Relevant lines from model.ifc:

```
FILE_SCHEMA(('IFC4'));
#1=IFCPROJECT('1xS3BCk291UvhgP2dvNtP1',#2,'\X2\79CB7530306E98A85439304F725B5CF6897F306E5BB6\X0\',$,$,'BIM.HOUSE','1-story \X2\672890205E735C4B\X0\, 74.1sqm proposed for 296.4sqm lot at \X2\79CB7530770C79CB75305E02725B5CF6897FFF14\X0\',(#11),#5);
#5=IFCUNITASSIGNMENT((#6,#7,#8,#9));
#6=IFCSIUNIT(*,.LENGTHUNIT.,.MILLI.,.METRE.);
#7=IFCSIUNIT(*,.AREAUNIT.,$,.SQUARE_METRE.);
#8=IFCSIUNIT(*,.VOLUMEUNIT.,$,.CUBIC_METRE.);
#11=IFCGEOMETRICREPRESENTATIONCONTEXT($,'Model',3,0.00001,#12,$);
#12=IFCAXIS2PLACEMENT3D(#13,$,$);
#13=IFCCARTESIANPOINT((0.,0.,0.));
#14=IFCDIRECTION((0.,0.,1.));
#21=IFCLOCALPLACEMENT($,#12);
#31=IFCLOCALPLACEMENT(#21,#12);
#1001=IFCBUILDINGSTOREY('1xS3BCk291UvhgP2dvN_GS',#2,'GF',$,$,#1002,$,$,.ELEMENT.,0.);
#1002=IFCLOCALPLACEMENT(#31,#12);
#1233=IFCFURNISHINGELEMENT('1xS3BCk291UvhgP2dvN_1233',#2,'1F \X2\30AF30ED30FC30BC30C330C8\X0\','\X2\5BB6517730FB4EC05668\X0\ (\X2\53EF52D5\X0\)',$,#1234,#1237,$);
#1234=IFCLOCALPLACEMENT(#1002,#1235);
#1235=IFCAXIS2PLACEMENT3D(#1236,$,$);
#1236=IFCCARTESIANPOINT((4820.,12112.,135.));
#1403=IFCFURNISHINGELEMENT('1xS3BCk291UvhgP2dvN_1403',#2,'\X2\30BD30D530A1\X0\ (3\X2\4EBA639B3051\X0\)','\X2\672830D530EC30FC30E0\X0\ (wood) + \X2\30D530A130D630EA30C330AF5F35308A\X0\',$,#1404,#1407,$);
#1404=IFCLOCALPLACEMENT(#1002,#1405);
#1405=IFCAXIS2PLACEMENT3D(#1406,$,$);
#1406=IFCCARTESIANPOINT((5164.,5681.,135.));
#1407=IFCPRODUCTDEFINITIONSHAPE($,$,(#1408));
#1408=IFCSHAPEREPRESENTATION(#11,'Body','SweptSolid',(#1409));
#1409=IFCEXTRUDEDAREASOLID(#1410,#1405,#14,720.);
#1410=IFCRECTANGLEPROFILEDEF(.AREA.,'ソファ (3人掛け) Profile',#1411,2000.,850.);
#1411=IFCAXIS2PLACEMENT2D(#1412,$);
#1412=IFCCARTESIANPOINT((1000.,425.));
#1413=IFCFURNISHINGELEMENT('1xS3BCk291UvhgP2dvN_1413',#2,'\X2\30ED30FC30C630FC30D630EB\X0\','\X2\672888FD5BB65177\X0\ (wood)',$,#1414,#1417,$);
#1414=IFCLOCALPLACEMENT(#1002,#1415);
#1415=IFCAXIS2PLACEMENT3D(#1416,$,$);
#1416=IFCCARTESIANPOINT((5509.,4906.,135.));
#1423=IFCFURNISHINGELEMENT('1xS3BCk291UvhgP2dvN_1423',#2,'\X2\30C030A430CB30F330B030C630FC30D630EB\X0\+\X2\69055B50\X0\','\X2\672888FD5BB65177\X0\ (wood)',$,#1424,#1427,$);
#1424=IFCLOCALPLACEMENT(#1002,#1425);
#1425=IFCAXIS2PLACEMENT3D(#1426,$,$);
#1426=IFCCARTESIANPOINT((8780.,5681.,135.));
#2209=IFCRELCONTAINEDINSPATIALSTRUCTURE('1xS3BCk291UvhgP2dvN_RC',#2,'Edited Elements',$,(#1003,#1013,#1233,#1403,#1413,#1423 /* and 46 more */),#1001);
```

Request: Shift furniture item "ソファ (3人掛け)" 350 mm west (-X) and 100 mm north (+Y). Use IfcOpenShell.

```python
import ifcopenshell
import ifcopenshell.api.geometry
import ifcopenshell.util.placement

model = ifcopenshell.open("model.ifc")

item = model.by_guid("1xS3BCk291UvhgP2dvN_1403")
matrix = ifcopenshell.util.placement.get_local_placement(item.ObjectPlacement)
matrix[0, 3] -= 350.0
matrix[1, 3] += 100.0
ifcopenshell.api.geometry.edit_object_placement(model, product=item, matrix=matrix, is_si=False)

print(ifcopenshell.util.placement.get_local_placement(item.ObjectPlacement).round(3) + 0.0)

model.write("model_rev.ifc")
```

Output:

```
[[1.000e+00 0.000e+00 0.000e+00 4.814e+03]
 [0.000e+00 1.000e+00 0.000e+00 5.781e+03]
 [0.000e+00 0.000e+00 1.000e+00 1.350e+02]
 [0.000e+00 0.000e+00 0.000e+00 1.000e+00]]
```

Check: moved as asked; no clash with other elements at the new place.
